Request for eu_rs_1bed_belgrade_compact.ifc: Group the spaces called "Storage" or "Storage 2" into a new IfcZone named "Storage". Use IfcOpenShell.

First a look at what the model holds.

```python
import ifcopenshell

model = ifcopenshell.open("eu_rs_1bed_belgrade_compact.ifc")
print(model.schema)
seen = {}
for space in model.by_type("IfcSpace"):
    seen[space.LongName] = seen.get(space.LongName, 0) + 1
for name, count in sorted(seen.items(), key=str):
    print(count, "x", name)
print("zones:", [z.Name for z in model.by_type("IfcZone")][:20])
```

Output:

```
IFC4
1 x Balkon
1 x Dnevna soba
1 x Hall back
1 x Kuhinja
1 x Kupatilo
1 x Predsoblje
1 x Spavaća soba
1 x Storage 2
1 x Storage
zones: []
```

```python
import ifcopenshell
import ifcopenshell.api.group
import ifcopenshell.api.root

model = ifcopenshell.open("eu_rs_1bed_belgrade_compact.ifc")

names = {"Storage", "Storage 2"}
spaces = [s for s in model.by_type("IfcSpace") if s.LongName in names]

zone = ifcopenshell.api.root.create_entity(model, ifc_class="IfcZone", name="Storage")
ifcopenshell.api.group.assign_group(model, products=spaces, group=zone)
print(len(spaces), "spaces in", zone.Name)

model.write("eu_rs_1bed_belgrade_compact-out.ifc")
```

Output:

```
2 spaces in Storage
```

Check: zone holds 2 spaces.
